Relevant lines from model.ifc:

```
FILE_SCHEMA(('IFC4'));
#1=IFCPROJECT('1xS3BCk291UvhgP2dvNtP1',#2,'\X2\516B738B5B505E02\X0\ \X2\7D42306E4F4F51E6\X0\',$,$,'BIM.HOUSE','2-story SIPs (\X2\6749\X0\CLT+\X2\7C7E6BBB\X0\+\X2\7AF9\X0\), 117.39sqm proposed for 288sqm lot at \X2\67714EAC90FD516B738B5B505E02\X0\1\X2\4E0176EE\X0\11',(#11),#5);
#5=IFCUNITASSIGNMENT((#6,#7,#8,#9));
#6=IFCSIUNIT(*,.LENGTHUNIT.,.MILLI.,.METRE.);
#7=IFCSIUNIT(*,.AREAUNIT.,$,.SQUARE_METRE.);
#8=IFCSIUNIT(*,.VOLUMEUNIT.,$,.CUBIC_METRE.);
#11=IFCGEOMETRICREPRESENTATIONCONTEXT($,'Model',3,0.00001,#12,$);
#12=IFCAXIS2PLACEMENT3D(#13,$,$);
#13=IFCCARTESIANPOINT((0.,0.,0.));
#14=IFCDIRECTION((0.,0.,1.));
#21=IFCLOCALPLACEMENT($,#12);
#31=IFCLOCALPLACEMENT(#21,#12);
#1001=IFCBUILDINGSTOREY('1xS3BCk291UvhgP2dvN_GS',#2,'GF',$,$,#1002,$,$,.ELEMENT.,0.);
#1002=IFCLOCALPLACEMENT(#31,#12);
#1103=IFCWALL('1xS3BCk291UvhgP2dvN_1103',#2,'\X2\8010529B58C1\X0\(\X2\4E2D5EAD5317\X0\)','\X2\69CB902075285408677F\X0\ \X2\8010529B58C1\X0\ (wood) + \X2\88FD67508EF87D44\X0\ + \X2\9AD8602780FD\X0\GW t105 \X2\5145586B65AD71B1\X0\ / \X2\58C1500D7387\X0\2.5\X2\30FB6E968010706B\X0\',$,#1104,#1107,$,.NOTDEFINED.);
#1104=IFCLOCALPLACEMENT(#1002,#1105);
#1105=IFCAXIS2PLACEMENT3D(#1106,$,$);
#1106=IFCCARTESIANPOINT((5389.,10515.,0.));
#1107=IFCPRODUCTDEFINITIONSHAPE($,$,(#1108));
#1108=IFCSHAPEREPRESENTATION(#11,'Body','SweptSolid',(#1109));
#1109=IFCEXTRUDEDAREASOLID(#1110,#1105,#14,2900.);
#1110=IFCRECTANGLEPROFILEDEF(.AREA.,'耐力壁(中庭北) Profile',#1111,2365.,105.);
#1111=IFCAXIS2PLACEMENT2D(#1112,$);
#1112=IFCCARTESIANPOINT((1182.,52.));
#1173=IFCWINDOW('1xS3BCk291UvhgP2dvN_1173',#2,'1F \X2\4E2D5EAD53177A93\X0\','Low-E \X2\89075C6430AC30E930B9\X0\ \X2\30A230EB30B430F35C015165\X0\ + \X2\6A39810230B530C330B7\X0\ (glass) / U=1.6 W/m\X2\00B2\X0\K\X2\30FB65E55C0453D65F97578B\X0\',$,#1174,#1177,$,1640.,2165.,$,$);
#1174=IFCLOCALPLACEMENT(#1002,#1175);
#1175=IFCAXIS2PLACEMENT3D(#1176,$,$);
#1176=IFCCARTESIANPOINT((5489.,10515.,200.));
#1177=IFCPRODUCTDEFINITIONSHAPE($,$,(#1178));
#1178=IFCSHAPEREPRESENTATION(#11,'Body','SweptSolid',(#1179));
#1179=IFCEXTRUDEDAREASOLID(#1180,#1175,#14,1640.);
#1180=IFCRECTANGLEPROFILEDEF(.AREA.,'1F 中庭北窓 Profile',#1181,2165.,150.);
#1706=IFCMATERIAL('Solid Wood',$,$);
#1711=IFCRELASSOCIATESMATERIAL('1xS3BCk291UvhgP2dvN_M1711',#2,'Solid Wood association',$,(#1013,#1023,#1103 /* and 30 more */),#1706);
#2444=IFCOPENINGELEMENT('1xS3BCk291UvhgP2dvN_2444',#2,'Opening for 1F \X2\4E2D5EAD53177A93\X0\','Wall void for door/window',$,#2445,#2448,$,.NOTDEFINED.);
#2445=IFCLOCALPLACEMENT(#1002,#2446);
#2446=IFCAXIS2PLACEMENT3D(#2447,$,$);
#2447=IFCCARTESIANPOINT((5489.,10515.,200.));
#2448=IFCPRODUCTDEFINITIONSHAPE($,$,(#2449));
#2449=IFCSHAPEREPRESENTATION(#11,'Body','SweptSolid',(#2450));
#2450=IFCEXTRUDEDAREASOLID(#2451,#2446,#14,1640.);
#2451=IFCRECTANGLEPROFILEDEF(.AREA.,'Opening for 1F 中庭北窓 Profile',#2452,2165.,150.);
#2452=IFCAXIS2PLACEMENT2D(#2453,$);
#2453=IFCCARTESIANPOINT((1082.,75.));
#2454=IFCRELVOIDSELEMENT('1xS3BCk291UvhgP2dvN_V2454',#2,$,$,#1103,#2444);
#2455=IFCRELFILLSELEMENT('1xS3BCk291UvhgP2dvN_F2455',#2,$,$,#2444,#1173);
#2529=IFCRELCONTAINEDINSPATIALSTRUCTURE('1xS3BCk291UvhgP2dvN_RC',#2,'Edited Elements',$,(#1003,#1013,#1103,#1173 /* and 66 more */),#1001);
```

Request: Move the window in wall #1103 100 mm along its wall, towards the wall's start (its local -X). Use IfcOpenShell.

```python
import ifcopenshell
import ifcopenshell.api.geometry
import ifcopenshell.util.placement
import ifcopenshell.util.unit

model = ifcopenshell.open("model.ifc")
unit_scale = ifcopenshell.util.unit.calculate_unit_scale(model)

window = model.by_guid("1xS3BCk291UvhgP2dvN_1173")
opening = window.FillsVoids[0].RelatingOpeningElement
wall = opening.VoidsElements[0].RelatingBuildingElement

wall_matrix = ifcopenshell.util.placement.get_local_placement(wall.ObjectPlacement)
shift = wall_matrix[:3, 0] * -0.1 / unit_scale
before = ifcopenshell.util.placement.get_local_placement(window.ObjectPlacement)[:3, 3].copy()

# The window is not placed relative to its opening, so move both.
for product in (opening, window):
    matrix = ifcopenshell.util.placement.get_local_placement(product.ObjectPlacement)
    matrix[:3, 3] += shift
    ifcopenshell.api.geometry.edit_object_placement(model, product=product, matrix=matrix, is_si=False)

after = ifcopenshell.util.placement.get_local_placement(window.ObjectPlacement)[:3, 3]
print("window moved by", (after - before).round(3) + 0.0)

model.write("model_rev.ifc")
```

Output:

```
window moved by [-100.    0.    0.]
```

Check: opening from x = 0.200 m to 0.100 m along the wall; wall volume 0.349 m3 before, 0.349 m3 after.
